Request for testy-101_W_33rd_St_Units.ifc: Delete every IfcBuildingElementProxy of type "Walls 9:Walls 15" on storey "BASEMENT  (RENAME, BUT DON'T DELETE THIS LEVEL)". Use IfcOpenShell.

First a look at what the model holds.

```python
import ifcopenshell
import ifcopenshell.util.element

model = ifcopenshell.open("testy-101_W_33rd_St_Units.ifc")
print(model.schema)
storey = next(s for s in model.by_type("IfcBuildingStorey") if s.Name == "BASEMENT  (RENAME, BUT DON'T DELETE THIS LEVEL)")
proxies = [e for e in ifcopenshell.util.element.get_decomposition(storey) if e.is_a("IfcBuildingElementProxy")]
seen = {}
for e in proxies:
    element_type = ifcopenshell.util.element.get_type(e)
    name = element_type.Name if element_type not in (None, e) else None
    seen[name] = seen.get(name, 0) + 1
for name, count in sorted(seen.items(), key=str):
    print(count, "x", name)
```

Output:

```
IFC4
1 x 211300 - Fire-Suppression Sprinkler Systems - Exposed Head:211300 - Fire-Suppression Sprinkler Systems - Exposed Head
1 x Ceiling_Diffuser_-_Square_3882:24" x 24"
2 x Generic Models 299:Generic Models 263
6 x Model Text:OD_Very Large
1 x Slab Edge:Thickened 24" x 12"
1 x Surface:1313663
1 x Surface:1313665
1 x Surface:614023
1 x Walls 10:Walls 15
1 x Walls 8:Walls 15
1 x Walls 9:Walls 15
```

```python
import ifcopenshell
import ifcopenshell.api.root
import ifcopenshell.util.element

model = ifcopenshell.open("testy-101_W_33rd_St_Units.ifc")

storey = next(s for s in model.by_type("IfcBuildingStorey") if s.Name == "BASEMENT  (RENAME, BUT DON'T DELETE THIS LEVEL)")
proxies = [e for e in ifcopenshell.util.element.get_decomposition(storey) if e.is_a("IfcBuildingElementProxy")]
targets = [e for e in proxies if (t := ifcopenshell.util.element.get_type(e)) not in (None, e) and t.Name == "Walls 9:Walls 15"]

for e in targets:
    ifcopenshell.api.root.remove_product(model, product=e)
print(len(targets), "removed")

model.write("testy-101_W_33rd_St_Units_edited.ifc")
```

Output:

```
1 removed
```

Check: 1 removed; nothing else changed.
